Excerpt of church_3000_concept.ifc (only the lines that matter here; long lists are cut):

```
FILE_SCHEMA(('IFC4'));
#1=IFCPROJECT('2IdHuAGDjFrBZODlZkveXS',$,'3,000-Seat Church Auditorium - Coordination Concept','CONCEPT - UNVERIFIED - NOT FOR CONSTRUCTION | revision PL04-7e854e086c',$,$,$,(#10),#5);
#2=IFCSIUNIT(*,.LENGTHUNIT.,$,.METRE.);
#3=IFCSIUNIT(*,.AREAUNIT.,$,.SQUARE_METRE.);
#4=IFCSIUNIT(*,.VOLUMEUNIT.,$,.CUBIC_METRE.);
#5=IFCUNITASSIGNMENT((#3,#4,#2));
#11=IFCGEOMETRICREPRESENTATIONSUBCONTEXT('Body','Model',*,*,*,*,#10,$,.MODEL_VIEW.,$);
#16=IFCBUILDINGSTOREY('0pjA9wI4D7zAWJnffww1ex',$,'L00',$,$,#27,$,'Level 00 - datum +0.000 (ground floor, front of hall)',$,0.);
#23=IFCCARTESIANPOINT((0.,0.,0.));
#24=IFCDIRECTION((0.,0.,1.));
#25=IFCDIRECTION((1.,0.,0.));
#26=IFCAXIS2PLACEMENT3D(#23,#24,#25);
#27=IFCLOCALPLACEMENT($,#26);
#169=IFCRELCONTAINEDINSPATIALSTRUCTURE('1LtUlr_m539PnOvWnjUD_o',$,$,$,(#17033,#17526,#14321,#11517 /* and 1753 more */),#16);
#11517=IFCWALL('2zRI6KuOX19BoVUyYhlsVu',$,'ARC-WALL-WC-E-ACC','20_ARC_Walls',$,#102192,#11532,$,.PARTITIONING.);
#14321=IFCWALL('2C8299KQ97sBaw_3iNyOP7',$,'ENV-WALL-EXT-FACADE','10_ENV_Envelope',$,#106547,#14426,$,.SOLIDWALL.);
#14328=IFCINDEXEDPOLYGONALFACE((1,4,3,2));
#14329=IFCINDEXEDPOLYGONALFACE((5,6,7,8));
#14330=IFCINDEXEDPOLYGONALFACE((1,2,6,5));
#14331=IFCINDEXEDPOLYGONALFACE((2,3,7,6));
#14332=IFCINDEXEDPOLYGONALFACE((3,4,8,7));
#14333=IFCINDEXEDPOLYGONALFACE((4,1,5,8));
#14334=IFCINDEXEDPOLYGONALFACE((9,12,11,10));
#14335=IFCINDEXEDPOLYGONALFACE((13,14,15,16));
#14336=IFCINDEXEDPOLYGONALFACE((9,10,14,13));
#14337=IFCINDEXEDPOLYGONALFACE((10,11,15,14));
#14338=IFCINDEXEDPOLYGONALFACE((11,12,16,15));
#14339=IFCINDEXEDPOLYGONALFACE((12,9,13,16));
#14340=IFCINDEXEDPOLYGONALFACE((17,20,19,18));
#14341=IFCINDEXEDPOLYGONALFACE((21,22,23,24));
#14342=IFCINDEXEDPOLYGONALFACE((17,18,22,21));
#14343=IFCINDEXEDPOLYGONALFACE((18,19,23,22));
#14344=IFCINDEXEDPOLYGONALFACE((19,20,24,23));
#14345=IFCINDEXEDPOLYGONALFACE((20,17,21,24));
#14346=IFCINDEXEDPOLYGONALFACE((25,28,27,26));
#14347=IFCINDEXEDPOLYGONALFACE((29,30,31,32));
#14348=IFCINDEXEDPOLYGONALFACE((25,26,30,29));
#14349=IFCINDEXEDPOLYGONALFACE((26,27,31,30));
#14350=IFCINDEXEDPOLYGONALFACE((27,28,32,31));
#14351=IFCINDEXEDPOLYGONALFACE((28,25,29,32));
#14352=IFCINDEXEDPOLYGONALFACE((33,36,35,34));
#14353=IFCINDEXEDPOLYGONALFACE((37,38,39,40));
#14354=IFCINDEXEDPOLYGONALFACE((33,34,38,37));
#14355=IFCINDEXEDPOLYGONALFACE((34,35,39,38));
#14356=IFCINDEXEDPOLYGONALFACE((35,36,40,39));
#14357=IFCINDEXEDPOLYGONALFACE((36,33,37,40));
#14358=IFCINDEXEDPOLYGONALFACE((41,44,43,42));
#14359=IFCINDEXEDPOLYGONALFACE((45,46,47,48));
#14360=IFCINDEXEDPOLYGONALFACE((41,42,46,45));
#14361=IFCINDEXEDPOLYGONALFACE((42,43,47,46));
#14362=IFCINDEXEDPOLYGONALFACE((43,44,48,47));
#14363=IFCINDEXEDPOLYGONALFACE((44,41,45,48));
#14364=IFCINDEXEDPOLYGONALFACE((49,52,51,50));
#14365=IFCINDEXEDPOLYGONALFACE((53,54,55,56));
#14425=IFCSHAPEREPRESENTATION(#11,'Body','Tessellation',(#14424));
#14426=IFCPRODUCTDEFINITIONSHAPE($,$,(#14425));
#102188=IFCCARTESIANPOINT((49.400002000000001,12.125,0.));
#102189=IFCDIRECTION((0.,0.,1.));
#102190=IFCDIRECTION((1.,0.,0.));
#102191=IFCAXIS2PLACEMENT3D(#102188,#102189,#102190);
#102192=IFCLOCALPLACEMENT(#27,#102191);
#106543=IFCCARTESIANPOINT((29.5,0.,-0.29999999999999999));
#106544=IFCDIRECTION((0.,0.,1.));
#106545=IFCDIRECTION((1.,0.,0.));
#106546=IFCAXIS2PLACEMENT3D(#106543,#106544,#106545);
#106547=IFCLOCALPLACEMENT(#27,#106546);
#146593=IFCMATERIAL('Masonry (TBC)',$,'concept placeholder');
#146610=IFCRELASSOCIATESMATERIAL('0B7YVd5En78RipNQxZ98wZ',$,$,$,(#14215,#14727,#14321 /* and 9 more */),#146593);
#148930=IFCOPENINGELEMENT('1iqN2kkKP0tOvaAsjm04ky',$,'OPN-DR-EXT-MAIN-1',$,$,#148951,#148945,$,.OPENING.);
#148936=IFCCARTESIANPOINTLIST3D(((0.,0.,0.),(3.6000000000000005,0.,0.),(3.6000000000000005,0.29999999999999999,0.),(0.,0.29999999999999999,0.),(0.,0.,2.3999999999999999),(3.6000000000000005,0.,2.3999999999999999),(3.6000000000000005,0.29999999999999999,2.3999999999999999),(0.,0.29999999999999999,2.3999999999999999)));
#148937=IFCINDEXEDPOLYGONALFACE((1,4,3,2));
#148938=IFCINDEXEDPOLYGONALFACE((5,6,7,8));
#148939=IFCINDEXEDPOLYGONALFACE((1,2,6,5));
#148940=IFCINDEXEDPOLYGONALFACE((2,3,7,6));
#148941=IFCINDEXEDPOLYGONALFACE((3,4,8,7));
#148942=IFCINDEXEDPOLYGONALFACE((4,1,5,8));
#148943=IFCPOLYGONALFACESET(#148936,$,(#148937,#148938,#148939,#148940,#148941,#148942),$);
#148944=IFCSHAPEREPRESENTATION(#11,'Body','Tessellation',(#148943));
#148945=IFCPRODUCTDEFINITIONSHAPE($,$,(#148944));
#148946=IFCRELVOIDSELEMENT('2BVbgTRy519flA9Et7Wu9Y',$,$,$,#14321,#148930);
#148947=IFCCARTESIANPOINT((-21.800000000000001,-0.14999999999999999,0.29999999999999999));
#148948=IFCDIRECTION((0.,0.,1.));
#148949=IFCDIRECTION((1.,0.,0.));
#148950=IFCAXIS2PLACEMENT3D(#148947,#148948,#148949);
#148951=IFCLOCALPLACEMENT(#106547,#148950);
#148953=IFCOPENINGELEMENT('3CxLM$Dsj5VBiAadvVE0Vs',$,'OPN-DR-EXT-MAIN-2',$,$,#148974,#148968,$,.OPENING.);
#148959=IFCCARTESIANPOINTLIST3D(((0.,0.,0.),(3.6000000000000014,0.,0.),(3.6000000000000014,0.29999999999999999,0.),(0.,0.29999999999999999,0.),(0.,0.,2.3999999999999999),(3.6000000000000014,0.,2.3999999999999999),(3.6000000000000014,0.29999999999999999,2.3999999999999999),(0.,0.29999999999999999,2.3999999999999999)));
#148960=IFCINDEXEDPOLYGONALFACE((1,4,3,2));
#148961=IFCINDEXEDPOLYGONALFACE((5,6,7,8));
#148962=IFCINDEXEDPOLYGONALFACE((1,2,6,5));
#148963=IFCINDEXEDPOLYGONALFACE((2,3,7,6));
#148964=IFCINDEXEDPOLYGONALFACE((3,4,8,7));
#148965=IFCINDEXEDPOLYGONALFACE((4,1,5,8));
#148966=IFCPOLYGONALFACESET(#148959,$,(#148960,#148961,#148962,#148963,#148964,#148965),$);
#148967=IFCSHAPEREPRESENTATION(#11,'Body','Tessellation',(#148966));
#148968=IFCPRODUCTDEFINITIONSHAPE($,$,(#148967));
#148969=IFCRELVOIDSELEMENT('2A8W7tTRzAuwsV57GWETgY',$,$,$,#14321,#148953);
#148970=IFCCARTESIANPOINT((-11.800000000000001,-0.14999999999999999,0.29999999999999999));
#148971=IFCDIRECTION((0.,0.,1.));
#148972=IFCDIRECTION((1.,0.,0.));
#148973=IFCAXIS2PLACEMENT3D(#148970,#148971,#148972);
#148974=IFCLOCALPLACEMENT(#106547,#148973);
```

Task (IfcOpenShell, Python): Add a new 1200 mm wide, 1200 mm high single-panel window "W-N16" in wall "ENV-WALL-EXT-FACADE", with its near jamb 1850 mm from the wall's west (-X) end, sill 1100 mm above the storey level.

```python
import numpy as np
import ifcopenshell
import ifcopenshell.api.feature
import ifcopenshell.api.geometry
import ifcopenshell.api.root
import ifcopenshell.api.spatial
import ifcopenshell.geom
import ifcopenshell.util.element
import ifcopenshell.util.placement
import ifcopenshell.util.representation
import ifcopenshell.util.shape
import ifcopenshell.util.unit

model = ifcopenshell.open("church_3000_concept.ifc")
unit_scale = ifcopenshell.util.unit.calculate_unit_scale(model)
settings = ifcopenshell.geom.settings()


def volume(element):
    """Net volume in cubic metres, openings subtracted."""
    shape = ifcopenshell.geom.create_shape(settings, element)
    return ifcopenshell.util.shape.get_volume(shape.geometry)


wall = model.by_id(14321)
storey = ifcopenshell.util.element.get_container(wall, ifc_class="IfcBuildingStorey")
context = ifcopenshell.util.representation.get_context(model, "Model", "Body", "MODEL_VIEW")
before = volume(wall)

width, height, from_end, sill = 1.2, 1.2, 1.85, 1.1  # metres

# The wall runs along its own X axis, and the end named is its -X end.
wall_shape = ifcopenshell.geom.create_shape(settings, wall)
x, y, z = ifcopenshell.util.shape.get_vertices(wall_shape.geometry).T
start = x.min() + from_end
face, thickness = float(y.min()), float(y.max() - y.min())
wall_matrix = ifcopenshell.util.placement.get_local_placement(wall.ObjectPlacement)
level = ifcopenshell.util.placement.get_local_placement(storey.ObjectPlacement)[2, 3]


def in_wall(x, y):
    """Placement at x, y metres in the wall's axes, at sill height."""
    matrix = wall_matrix.copy()
    matrix[:, 3] = wall_matrix @ np.array([x / unit_scale, y / unit_scale, 0.0, 1.0])
    matrix[2, 3] = level + sill / unit_scale
    return matrix


# Opening: a box that overshoots both wall faces by 50 mm.
opening = ifcopenshell.api.root.create_entity(model, ifc_class="IfcOpeningElement", predefined_type="OPENING")
box = ifcopenshell.api.geometry.add_wall_representation(
    model, context=context, length=width, height=height, thickness=thickness + 0.1
)
ifcopenshell.api.geometry.assign_representation(model, product=opening, representation=box)
ifcopenshell.api.geometry.edit_object_placement(model, product=opening, matrix=in_wall(start, face - 0.05), is_si=False)
ifcopenshell.api.feature.add_feature(model, feature=opening, element=wall)

window = ifcopenshell.api.root.create_entity(model, ifc_class="IfcWindow", name="W-N16", predefined_type="WINDOW")
window.OverallWidth, window.OverallHeight = width / unit_scale, height / unit_scale
window.PartitioningType = "SINGLE_PANEL"
body = ifcopenshell.api.geometry.add_window_representation(
    model,
    context=context,
    overall_width=window.OverallWidth,
    overall_height=window.OverallHeight,
    partition_type="SINGLE_PANEL",
)
ifcopenshell.api.geometry.assign_representation(model, product=window, representation=body)
ifcopenshell.api.spatial.assign_container(model, products=[window], relating_structure=storey)
ifcopenshell.api.feature.add_filling(model, opening=opening, element=window)

# Centre the window in the wall's thickness.
ifcopenshell.api.geometry.edit_object_placement(model, product=window, matrix=in_wall(start, face), is_si=False)
window_shape = ifcopenshell.geom.create_shape(settings, window)
depth = ifcopenshell.util.shape.get_vertices(window_shape.geometry)[:, 1]
offset = face + thickness / 2 - (depth.min() + depth.max()) / 2
ifcopenshell.api.geometry.edit_object_placement(model, product=window, matrix=in_wall(start, offset), is_si=False)

after = volume(wall)

print(f"wall volume {before:.3f} -> {after:.3f} m3")

model.write("church_3000_concept_edited.ifc")
```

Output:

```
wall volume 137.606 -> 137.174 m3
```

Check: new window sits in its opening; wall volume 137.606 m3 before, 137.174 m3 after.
